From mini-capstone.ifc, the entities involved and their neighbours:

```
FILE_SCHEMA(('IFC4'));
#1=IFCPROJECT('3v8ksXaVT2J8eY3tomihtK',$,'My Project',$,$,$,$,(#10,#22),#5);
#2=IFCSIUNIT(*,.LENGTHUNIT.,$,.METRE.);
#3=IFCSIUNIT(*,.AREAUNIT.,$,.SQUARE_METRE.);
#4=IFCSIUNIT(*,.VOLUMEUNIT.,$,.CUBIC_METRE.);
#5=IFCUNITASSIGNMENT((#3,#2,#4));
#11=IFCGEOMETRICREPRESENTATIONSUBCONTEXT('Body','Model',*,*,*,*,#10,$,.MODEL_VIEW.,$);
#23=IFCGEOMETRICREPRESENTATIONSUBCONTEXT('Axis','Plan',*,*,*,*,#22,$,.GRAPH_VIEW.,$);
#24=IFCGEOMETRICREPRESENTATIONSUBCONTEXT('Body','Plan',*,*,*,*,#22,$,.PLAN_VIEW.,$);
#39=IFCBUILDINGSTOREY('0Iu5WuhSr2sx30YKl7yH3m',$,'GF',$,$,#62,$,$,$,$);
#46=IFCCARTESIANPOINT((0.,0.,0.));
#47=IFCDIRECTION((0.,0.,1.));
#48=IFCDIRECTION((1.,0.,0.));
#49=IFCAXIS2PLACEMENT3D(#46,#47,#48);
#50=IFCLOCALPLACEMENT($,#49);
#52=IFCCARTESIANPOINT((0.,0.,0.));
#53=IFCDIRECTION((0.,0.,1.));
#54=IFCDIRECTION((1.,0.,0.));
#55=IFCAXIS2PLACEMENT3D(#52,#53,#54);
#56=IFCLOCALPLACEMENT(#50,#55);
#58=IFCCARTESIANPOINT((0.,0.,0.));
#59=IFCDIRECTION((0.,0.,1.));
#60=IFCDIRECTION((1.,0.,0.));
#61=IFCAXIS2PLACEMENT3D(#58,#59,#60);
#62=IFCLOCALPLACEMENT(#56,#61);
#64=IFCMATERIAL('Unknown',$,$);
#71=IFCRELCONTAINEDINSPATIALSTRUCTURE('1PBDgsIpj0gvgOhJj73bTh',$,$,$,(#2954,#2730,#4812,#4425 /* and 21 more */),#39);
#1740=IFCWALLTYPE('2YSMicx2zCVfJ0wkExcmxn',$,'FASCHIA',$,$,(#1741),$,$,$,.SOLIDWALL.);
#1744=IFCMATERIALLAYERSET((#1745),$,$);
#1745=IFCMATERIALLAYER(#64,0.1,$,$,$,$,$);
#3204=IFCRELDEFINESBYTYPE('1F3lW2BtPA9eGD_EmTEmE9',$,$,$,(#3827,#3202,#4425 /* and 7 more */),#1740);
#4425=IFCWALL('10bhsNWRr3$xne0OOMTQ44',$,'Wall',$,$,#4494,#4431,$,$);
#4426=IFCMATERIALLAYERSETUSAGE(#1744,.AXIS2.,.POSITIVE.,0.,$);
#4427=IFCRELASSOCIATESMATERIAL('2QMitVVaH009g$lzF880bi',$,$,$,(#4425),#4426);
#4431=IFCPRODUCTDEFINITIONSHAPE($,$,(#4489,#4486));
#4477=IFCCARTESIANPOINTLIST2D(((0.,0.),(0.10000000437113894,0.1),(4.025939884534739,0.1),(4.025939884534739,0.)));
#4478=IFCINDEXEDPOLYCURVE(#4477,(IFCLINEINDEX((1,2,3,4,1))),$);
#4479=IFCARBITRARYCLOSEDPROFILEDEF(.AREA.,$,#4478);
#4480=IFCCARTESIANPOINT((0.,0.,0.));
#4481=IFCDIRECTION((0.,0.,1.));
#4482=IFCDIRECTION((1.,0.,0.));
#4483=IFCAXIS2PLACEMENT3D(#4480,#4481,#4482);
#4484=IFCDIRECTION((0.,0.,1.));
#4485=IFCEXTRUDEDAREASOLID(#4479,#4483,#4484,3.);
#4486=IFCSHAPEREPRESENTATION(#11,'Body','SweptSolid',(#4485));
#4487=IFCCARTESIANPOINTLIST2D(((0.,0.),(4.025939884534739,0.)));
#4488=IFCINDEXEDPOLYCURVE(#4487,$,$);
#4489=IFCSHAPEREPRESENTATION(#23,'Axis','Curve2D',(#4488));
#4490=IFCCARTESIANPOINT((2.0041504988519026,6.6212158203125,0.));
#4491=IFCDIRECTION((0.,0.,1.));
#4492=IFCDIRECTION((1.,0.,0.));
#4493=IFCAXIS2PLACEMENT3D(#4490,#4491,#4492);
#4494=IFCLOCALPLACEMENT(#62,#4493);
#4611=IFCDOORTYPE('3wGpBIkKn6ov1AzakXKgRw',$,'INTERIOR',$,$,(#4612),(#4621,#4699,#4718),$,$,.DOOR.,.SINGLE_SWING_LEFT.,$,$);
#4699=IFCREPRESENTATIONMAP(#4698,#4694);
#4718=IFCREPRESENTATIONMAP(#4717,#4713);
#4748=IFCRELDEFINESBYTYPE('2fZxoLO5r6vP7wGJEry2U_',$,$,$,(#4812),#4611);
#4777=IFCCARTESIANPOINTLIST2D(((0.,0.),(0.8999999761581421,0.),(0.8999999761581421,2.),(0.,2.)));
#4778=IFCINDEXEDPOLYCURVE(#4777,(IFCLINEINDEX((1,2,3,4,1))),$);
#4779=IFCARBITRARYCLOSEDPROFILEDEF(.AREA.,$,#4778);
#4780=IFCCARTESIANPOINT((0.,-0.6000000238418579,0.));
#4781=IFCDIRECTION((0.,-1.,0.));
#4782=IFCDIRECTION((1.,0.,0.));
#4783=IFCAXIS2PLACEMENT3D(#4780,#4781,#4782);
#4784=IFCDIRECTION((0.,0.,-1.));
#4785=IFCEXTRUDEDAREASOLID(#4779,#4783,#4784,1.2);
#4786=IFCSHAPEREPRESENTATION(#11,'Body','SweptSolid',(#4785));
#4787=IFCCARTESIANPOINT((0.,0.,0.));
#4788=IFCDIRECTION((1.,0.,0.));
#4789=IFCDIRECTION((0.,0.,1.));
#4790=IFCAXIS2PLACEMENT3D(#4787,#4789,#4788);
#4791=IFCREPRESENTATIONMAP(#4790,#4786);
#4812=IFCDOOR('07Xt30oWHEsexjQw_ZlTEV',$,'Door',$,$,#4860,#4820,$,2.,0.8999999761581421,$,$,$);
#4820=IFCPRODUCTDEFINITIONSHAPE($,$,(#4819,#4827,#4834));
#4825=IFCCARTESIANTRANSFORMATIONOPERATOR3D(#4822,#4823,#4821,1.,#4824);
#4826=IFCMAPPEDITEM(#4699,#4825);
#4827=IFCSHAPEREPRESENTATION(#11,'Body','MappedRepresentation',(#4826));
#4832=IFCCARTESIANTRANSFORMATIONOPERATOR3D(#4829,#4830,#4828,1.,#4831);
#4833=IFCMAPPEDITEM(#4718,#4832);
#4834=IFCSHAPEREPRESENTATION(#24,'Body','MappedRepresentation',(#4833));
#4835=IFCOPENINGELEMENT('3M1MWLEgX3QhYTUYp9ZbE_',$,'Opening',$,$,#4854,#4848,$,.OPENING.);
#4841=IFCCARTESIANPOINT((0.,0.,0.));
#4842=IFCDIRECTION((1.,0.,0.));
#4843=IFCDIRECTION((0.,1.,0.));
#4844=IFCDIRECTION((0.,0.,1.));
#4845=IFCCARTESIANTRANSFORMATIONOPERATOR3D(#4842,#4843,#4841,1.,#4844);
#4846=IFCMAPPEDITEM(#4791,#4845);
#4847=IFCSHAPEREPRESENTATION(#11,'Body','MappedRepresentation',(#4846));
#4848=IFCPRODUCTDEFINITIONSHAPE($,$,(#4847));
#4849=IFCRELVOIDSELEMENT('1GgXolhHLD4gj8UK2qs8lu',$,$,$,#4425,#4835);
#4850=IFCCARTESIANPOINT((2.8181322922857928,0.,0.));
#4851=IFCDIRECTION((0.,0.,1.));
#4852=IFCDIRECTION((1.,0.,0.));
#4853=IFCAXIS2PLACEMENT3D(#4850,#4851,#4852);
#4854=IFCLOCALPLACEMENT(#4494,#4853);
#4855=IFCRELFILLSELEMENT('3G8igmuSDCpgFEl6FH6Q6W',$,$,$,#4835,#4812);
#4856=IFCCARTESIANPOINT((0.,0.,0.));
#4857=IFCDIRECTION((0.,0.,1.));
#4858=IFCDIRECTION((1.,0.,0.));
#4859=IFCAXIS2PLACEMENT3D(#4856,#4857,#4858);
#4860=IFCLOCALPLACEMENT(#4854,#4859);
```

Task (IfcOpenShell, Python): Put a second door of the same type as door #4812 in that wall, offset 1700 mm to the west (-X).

```python
import ifcopenshell
import ifcopenshell.api.feature
import ifcopenshell.api.geometry
import ifcopenshell.api.root
import ifcopenshell.geom
import ifcopenshell.util.element
import ifcopenshell.util.placement
import ifcopenshell.util.shape

model = ifcopenshell.open("mini-capstone.ifc")
settings = ifcopenshell.geom.settings()


def volume(element):
    """Net volume in cubic metres, openings subtracted."""
    shape = ifcopenshell.geom.create_shape(settings, element)
    return ifcopenshell.util.shape.get_volume(shape.geometry)


door = model.by_id(4812)
opening = door.FillsVoids[0].RelatingOpeningElement
wall = opening.VoidsElements[0].RelatingBuildingElement
before = volume(wall)
shift = ifcopenshell.util.placement.get_local_placement(wall.ObjectPlacement)[:3, 0] * -1.7

# copy_class copies the void relationship, type, container and properties, but no geometry.
new_opening = ifcopenshell.api.root.copy_class(model, product=opening)
new_opening.Representation = ifcopenshell.util.element.copy_deep(
    model, opening.Representation, exclude=["IfcGeometricRepresentationContext", "IfcRepresentationMap"]
)
new_door = ifcopenshell.api.root.copy_class(model, product=door)
new_door.Representation = ifcopenshell.util.element.copy_deep(
    model, door.Representation, exclude=["IfcGeometricRepresentationContext", "IfcRepresentationMap"]
)
ifcopenshell.api.feature.add_filling(model, opening=new_opening, element=new_door)

for old, new in ((opening, new_opening), (door, new_door)):
    matrix = ifcopenshell.util.placement.get_local_placement(old.ObjectPlacement)
    matrix[:3, 3] += shift
    ifcopenshell.api.geometry.edit_object_placement(model, product=new, matrix=matrix, is_si=False)

after = volume(wall)

print(f"wall volume {before:.3f} -> {after:.3f} m3")

model.write("mini-capstone_edited.ifc")
```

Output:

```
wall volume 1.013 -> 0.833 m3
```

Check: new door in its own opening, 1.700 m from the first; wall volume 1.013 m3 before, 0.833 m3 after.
